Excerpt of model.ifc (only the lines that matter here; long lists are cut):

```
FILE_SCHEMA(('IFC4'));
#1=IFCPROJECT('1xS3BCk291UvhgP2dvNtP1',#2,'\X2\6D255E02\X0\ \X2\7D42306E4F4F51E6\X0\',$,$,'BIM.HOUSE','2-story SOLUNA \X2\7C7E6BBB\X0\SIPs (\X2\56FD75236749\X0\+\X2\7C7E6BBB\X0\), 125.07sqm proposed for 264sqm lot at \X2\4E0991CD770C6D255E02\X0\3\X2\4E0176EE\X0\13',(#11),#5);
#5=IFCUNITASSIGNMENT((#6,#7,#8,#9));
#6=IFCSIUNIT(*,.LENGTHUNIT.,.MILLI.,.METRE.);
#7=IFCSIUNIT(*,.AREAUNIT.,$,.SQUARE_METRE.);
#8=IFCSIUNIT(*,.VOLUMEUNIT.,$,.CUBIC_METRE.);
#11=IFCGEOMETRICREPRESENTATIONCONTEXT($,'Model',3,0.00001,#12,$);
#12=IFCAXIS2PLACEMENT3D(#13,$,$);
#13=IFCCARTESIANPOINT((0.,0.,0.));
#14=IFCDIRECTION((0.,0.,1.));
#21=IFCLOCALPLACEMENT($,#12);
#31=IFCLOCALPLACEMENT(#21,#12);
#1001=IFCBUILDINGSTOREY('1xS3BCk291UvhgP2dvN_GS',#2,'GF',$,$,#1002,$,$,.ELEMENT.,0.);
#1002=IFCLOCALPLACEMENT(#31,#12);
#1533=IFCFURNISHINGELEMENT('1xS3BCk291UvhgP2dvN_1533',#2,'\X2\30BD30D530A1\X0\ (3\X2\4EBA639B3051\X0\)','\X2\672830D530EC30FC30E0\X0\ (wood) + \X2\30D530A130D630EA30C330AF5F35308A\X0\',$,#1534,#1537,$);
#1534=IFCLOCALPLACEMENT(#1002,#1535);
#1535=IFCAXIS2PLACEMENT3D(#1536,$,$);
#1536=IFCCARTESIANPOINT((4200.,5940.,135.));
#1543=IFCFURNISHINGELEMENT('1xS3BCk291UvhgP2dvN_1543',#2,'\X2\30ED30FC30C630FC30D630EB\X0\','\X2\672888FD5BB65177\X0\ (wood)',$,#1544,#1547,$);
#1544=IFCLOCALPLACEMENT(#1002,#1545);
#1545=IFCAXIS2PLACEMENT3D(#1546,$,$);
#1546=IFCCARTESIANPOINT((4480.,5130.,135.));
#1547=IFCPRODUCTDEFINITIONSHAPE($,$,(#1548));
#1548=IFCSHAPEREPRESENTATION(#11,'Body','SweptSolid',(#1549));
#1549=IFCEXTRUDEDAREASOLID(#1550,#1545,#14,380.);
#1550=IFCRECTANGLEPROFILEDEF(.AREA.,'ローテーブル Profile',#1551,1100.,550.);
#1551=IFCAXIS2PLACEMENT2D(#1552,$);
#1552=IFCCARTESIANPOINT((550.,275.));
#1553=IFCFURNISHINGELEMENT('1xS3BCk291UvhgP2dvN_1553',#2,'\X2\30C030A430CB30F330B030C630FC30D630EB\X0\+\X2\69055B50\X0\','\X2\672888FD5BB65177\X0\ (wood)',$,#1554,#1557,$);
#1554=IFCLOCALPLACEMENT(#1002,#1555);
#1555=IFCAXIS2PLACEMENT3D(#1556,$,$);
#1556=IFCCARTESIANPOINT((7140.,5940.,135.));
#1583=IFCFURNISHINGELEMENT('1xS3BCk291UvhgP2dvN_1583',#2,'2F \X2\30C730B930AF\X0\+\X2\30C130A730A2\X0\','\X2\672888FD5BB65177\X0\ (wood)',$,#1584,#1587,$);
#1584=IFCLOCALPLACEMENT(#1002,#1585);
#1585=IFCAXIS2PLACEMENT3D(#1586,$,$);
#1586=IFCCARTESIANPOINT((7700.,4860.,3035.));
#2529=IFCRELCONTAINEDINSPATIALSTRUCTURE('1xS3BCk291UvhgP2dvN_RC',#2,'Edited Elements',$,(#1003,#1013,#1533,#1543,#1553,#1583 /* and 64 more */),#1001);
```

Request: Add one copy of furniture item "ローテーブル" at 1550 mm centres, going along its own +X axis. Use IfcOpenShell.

```python
import ifcopenshell
import ifcopenshell.api.geometry
import ifcopenshell.api.root
import ifcopenshell.util.element
import ifcopenshell.util.placement
import ifcopenshell.util.unit

model = ifcopenshell.open("model.ifc")
unit_scale = ifcopenshell.util.unit.calculate_unit_scale(model)


def reuse_history(source, copy):
    """copy_class also copies each property set's owner history, people and application; keep the originals."""
    for rel in copy.IsDefinedBy:
        if rel.is_a("IfcRelDefinesByProperties") and (history := rel.RelatingPropertyDefinition.OwnerHistory):
            rel.RelatingPropertyDefinition.OwnerHistory = source.OwnerHistory
            ifcopenshell.util.element.remove_deep2(model, history)


source = model.by_id(1543)
base = ifcopenshell.util.placement.get_local_placement(source.ObjectPlacement)
step = base[:3, 0] * 1.55 / unit_scale

for i in range(1, 2):
    copy = ifcopenshell.api.root.copy_class(model, product=source)
    copy.Representation = ifcopenshell.util.element.copy_deep(
        model, source.Representation, exclude=["IfcGeometricRepresentationContext", "IfcRepresentationMap"]
    )
    reuse_history(source, copy)
    matrix = base.copy()
    matrix[:3, 3] += i * step
    print("added at", matrix[:3, 3].round(3) + 0.0)
    ifcopenshell.api.geometry.edit_object_placement(model, product=copy, matrix=matrix, is_si=False)

model.write("model_edited.ifc")
```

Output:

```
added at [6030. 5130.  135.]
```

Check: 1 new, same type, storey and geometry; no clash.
